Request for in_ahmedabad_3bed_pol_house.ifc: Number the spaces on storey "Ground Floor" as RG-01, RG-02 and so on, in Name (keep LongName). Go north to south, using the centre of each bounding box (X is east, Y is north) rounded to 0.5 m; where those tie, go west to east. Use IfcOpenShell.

First a look at what the model holds.

```python
import ifcopenshell
import ifcopenshell.util.element
import ifcopenshell.util.placement

model = ifcopenshell.open("in_ahmedabad_3bed_pol_house.ifc")
print(model.schema)
storey = next(s for s in model.by_type("IfcBuildingStorey") if s.Name == "Ground Floor")
spaces = [e for e in ifcopenshell.util.element.get_decomposition(storey) if e.is_a("IfcSpace")]
for e in sorted(spaces, key=lambda e: e.id()):
    origin = ifcopenshell.util.placement.get_local_placement(e.ObjectPlacement)[:3, 3]
    print(e.id(), e.Name, e.LongName, origin.round(2) + 0.0, sep=" | ")
```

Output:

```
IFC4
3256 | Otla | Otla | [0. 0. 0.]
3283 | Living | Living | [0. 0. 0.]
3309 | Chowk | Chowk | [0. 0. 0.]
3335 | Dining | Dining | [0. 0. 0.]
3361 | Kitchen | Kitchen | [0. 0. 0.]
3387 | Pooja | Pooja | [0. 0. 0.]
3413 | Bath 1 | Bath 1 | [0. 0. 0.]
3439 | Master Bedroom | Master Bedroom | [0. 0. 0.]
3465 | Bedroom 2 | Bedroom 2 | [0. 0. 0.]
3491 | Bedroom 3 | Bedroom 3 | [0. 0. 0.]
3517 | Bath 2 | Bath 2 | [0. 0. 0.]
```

```python
import ifcopenshell
import ifcopenshell.geom
import ifcopenshell.util.element
import ifcopenshell.util.shape

model = ifcopenshell.open("in_ahmedabad_3bed_pol_house.ifc")
settings = ifcopenshell.geom.settings()
settings.set("use-world-coords", True)


def centre(element):
    shape = ifcopenshell.geom.create_shape(settings, element)
    return ifcopenshell.util.shape.get_bbox_centroid(shape.geometry)


storey = next(s for s in model.by_type("IfcBuildingStorey") if s.Name == "Ground Floor")
spaces = [e for e in ifcopenshell.util.element.get_decomposition(storey) if e.is_a("IfcSpace")]

# Insertion points can sit at a corner or the storey origin, so sort by the geometry (in metres).
centres = {e: centre(e) for e in spaces}
spaces.sort(key=lambda e: (-round(centres[e][1] / 0.5), centres[e][0]))

for i, e in enumerate(spaces, start=1):
    number = f"RG-{i:02d}"
    e.Name = number
    print(e.id(), number)

model.write("in_ahmedabad_3bed_pol_house_v2.ifc")
```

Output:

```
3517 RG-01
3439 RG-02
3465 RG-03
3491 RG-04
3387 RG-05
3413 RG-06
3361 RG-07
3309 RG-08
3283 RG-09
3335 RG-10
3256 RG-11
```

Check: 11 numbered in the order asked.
